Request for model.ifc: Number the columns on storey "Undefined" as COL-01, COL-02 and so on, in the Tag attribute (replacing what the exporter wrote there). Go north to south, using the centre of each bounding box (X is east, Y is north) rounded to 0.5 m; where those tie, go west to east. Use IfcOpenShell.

First a look at what the model holds.

```python
import ifcopenshell
import ifcopenshell.util.element
import ifcopenshell.util.placement

model = ifcopenshell.open("model.ifc")
print(model.schema)
storey = next(s for s in model.by_type("IfcBuildingStorey") if s.Name == "Undefined")
columns = [e for e in ifcopenshell.util.element.get_decomposition(storey) if e.is_a("IfcColumn")]
for e in sorted(columns, key=lambda e: e.id()):
    origin = ifcopenshell.util.placement.get_local_placement(e.ObjectPlacement)[:3, 3]
    print(e.id(), e.Tag, e.Name, origin.round(2) + 0.0, sep=" | ")
```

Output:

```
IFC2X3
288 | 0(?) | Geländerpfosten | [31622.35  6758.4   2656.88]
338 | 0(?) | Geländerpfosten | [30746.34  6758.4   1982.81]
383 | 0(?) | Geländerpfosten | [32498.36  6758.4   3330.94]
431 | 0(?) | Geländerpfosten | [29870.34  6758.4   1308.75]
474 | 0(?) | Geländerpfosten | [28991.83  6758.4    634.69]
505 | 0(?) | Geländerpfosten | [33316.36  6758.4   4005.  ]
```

```python
import ifcopenshell
import ifcopenshell.geom
import ifcopenshell.util.element
import ifcopenshell.util.shape

model = ifcopenshell.open("model.ifc")
settings = ifcopenshell.geom.settings()
settings.set("use-world-coords", True)


def centre(element):
    shape = ifcopenshell.geom.create_shape(settings, element)
    return ifcopenshell.util.shape.get_bbox_centroid(shape.geometry)


storey = next(s for s in model.by_type("IfcBuildingStorey") if s.Name == "Undefined")
columns = [e for e in ifcopenshell.util.element.get_decomposition(storey) if e.is_a("IfcColumn")]

# Insertion points can sit at a corner or the storey origin, so sort by the geometry (in metres).
centres = {e: centre(e) for e in columns}
columns.sort(key=lambda e: (-round(centres[e][1] / 0.5), centres[e][0]))

for i, e in enumerate(columns, start=1):
    number = f"COL-{i:02d}"
    e.Tag = number
    print(e.id(), number)

model.write("model_updated.ifc")
```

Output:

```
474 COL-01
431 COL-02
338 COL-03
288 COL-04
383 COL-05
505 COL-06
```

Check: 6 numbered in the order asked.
